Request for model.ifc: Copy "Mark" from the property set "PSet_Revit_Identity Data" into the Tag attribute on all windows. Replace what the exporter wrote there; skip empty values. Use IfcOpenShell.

First a look at what the model holds.

```python
import ifcopenshell
import ifcopenshell.util.element

model = ifcopenshell.open("model.ifc")
print(model.schema)
windows = model.by_type("IfcWindow")
print(len(windows), "windows")
for e in windows[:8]:
    source = ifcopenshell.util.element.get_pset(e, "PSet_Revit_Identity Data", "Mark")
    target = e.Tag
    print(e.id(), repr(source), repr(target), sep=" | ")
```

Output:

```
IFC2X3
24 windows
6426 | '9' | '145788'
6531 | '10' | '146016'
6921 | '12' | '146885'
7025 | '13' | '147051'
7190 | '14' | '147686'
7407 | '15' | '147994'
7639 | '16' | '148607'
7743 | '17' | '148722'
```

```python
import ifcopenshell
import ifcopenshell.util.element

model = ifcopenshell.open("model.ifc")

count = 0
for e in model.by_type("IfcWindow"):
    value = ifcopenshell.util.element.get_pset(e, "PSet_Revit_Identity Data", "Mark")
    current = e.Tag
    if not value or not value.strip() or current == value:
        continue
    e.Tag = value
    count += 1

print(count, "windows updated")

model.write("model_v2.ifc")
```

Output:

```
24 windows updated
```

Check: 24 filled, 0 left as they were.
